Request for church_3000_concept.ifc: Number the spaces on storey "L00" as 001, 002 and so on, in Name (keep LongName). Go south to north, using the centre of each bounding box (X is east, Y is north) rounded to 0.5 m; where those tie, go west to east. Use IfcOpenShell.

First a look at what the model holds.

```python
import ifcopenshell
import ifcopenshell.util.element
import ifcopenshell.util.placement

model = ifcopenshell.open("church_3000_concept.ifc")
print(model.schema)
storey = next(s for s in model.by_type("IfcBuildingStorey") if s.Name == "L00")
spaces = [e for e in ifcopenshell.util.element.get_decomposition(storey) if e.is_a("IfcSpace")]
for e in sorted(spaces, key=lambda e: e.id()):
    origin = ifcopenshell.util.placement.get_local_placement(e.ObjectPlacement)[:3, 3]
    print(e.id(), e.Name, e.LongName, origin.round(2) + 0.0, sep=" | ")
```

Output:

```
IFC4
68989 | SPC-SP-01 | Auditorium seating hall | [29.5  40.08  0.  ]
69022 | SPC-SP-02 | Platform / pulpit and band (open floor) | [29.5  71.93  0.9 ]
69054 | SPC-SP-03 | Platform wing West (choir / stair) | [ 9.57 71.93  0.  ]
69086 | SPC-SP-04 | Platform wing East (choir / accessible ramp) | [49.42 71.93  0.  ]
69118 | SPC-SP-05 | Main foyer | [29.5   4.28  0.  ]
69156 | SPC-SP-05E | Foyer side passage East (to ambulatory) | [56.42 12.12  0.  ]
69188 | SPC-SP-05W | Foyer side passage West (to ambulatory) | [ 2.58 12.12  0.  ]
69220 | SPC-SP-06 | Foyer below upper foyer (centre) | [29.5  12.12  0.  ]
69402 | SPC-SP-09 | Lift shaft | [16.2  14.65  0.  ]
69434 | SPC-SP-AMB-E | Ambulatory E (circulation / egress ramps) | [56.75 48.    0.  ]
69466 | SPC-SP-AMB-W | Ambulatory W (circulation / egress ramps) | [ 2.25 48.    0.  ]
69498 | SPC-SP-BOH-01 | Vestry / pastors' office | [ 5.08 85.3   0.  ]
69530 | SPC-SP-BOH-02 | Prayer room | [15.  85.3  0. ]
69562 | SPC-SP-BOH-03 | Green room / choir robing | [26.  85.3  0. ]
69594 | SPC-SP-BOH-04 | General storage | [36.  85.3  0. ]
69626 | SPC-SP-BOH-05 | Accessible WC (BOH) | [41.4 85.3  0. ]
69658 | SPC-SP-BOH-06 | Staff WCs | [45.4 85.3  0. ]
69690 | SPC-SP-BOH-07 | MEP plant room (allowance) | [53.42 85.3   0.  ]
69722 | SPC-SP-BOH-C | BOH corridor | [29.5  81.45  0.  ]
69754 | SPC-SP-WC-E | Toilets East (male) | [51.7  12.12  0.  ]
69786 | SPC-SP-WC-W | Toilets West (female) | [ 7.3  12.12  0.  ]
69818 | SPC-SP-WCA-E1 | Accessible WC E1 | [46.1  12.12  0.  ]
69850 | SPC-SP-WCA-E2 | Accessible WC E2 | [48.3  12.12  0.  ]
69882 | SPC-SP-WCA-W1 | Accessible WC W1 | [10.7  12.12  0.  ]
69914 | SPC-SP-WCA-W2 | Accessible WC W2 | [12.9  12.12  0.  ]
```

```python
import ifcopenshell
import ifcopenshell.geom
import ifcopenshell.util.element
import ifcopenshell.util.shape

model = ifcopenshell.open("church_3000_concept.ifc")
settings = ifcopenshell.geom.settings()
settings.set("use-world-coords", True)


def centre(element):
    shape = ifcopenshell.geom.create_shape(settings, element)
    return ifcopenshell.util.shape.get_bbox_centroid(shape.geometry)


storey = next(s for s in model.by_type("IfcBuildingStorey") if s.Name == "L00")
spaces = [e for e in ifcopenshell.util.element.get_decomposition(storey) if e.is_a("IfcSpace")]

# Insertion points can sit at a corner or the storey origin, so sort by the geometry (in metres).
centres = {e: centre(e) for e in spaces}
spaces.sort(key=lambda e: (round(centres[e][1] / 0.5), centres[e][0]))

for i, e in enumerate(spaces, start=1):
    number = f"0{i:02d}"
    e.Name = number
    print(e.id(), number)

model.write("church_3000_concept_edited.ifc")
```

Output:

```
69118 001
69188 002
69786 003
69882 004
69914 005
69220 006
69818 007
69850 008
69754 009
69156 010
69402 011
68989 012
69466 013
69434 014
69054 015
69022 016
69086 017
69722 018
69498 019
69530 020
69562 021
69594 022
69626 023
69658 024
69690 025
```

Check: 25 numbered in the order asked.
